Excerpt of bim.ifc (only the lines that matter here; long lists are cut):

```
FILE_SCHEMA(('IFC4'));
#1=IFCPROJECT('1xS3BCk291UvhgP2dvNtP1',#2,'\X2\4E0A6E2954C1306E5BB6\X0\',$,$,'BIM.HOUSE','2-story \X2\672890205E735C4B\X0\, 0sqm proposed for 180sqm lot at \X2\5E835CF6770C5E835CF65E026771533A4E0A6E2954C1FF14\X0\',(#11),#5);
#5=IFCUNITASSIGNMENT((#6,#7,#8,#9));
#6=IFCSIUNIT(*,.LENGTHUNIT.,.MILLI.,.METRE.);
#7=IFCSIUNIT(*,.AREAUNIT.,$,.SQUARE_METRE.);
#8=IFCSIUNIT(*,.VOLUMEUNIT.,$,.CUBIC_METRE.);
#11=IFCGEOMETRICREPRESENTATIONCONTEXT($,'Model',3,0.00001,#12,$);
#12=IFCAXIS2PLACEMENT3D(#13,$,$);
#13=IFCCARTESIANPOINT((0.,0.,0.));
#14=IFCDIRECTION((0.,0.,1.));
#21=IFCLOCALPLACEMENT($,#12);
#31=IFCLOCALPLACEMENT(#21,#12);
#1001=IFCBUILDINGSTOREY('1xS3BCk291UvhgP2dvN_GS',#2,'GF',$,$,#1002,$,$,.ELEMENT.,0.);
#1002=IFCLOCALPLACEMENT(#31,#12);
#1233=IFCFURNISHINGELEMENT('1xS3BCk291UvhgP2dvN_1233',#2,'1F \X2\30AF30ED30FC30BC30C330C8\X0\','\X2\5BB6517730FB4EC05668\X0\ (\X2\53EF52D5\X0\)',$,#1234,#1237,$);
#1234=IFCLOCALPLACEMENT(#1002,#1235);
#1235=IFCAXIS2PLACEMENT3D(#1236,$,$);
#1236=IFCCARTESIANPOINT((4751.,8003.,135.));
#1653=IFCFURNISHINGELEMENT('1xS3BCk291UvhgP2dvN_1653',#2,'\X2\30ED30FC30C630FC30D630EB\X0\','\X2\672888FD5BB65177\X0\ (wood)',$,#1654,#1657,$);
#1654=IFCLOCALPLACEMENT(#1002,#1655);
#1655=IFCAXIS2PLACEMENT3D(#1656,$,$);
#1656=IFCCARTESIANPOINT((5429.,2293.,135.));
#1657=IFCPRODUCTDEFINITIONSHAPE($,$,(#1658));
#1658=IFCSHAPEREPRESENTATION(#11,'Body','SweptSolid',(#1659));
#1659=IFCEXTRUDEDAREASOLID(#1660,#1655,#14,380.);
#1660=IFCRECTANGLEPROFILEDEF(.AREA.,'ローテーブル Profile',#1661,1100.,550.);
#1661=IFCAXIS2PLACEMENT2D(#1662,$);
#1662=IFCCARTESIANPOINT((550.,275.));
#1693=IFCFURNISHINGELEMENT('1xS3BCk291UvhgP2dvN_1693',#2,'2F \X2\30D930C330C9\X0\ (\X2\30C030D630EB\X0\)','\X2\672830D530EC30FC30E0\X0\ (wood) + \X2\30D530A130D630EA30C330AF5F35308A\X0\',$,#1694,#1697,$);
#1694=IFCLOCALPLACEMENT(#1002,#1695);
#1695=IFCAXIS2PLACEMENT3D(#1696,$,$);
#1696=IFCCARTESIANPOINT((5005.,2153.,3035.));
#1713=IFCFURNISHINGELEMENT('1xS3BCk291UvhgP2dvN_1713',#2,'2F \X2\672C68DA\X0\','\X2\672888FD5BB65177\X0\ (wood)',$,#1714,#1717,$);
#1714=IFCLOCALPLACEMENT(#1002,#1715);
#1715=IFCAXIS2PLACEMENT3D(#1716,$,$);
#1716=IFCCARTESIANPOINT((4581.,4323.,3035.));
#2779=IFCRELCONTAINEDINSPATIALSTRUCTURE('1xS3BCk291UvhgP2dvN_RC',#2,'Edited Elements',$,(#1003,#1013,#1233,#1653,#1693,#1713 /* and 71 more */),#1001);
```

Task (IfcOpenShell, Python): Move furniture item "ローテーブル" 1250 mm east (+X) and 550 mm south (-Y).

```python
import ifcopenshell
import ifcopenshell.api.geometry
import ifcopenshell.util.placement

model = ifcopenshell.open("bim.ifc")

item = model.by_guid("1xS3BCk291UvhgP2dvN_1653")
matrix = ifcopenshell.util.placement.get_local_placement(item.ObjectPlacement)
matrix[0, 3] += 1250.0
matrix[1, 3] -= 550.0
ifcopenshell.api.geometry.edit_object_placement(model, product=item, matrix=matrix, is_si=False)

print(ifcopenshell.util.placement.get_local_placement(item.ObjectPlacement).round(3) + 0.0)

model.write("bim-out.ifc")
```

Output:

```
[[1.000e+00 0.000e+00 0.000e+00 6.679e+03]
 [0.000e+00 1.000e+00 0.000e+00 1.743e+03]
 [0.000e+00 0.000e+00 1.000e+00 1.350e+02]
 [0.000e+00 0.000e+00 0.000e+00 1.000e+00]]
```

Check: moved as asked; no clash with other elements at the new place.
